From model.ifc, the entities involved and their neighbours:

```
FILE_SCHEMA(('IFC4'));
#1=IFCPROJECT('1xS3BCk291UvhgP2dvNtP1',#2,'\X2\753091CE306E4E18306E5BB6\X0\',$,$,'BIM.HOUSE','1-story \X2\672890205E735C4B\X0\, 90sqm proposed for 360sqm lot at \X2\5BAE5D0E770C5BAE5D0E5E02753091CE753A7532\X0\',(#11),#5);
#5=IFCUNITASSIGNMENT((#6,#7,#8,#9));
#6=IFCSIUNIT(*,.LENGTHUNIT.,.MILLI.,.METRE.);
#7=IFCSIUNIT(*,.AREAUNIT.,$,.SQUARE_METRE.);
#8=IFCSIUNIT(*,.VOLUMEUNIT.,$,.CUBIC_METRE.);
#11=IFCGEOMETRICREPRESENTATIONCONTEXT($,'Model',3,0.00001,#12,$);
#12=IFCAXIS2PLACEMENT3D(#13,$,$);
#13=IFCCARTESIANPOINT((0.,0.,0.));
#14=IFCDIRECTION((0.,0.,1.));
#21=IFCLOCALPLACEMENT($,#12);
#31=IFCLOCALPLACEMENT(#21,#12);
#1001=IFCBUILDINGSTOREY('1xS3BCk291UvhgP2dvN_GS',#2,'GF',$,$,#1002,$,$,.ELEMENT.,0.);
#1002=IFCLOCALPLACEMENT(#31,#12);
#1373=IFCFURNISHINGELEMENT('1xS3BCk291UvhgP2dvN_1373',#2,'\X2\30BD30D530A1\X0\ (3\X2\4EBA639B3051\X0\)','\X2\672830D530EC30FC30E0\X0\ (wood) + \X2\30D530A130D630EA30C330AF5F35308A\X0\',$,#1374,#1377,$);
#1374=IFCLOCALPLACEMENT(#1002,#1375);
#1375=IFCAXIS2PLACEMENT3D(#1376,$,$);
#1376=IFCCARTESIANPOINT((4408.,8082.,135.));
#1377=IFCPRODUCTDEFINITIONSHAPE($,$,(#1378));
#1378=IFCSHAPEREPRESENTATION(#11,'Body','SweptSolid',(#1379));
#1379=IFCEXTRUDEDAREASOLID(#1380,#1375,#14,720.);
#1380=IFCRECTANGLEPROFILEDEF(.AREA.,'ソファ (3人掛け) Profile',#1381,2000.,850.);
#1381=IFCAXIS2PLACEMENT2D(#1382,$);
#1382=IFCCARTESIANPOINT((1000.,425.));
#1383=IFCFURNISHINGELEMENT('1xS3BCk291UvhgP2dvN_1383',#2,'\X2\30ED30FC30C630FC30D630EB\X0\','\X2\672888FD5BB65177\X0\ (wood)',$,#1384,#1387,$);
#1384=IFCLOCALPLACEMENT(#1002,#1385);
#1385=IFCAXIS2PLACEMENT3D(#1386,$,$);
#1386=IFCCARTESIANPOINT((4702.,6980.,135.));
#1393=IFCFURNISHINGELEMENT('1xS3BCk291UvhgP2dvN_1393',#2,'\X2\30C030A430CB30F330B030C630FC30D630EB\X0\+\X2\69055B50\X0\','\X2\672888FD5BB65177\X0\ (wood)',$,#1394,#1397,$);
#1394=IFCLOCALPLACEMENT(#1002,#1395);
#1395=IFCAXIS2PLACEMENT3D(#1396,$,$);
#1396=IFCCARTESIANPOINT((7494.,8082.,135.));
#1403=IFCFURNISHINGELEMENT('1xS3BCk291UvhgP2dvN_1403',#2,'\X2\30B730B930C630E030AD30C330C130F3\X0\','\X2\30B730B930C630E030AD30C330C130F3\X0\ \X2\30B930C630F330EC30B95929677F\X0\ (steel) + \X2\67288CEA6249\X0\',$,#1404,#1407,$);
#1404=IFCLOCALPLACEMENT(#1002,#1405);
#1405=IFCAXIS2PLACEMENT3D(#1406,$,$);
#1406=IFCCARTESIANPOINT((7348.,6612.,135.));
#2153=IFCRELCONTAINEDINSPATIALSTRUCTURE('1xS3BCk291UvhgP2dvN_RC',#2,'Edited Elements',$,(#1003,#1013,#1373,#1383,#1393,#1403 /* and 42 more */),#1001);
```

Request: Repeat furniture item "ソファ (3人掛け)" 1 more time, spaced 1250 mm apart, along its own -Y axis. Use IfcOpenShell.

```python
import ifcopenshell
import ifcopenshell.api.geometry
import ifcopenshell.api.root
import ifcopenshell.util.element
import ifcopenshell.util.placement
import ifcopenshell.util.unit

model = ifcopenshell.open("model.ifc")
unit_scale = ifcopenshell.util.unit.calculate_unit_scale(model)


def reuse_history(source, copy):
    """copy_class also copies each property set's owner history, people and application; keep the originals."""
    for rel in copy.IsDefinedBy:
        if rel.is_a("IfcRelDefinesByProperties") and (history := rel.RelatingPropertyDefinition.OwnerHistory):
            rel.RelatingPropertyDefinition.OwnerHistory = source.OwnerHistory
            ifcopenshell.util.element.remove_deep2(model, history)


source = model.by_guid("1xS3BCk291UvhgP2dvN_1373")
base = ifcopenshell.util.placement.get_local_placement(source.ObjectPlacement)
step = -base[:3, 1] * 1.25 / unit_scale

for i in range(1, 2):
    copy = ifcopenshell.api.root.copy_class(model, product=source)
    copy.Representation = ifcopenshell.util.element.copy_deep(
        model, source.Representation, exclude=["IfcGeometricRepresentationContext", "IfcRepresentationMap"]
    )
    reuse_history(source, copy)
    matrix = base.copy()
    matrix[:3, 3] += i * step
    print("added at", matrix[:3, 3].round(3) + 0.0)
    ifcopenshell.api.geometry.edit_object_placement(model, product=copy, matrix=matrix, is_si=False)

model.write("model_rev.ifc")
```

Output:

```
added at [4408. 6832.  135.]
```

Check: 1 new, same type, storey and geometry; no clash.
